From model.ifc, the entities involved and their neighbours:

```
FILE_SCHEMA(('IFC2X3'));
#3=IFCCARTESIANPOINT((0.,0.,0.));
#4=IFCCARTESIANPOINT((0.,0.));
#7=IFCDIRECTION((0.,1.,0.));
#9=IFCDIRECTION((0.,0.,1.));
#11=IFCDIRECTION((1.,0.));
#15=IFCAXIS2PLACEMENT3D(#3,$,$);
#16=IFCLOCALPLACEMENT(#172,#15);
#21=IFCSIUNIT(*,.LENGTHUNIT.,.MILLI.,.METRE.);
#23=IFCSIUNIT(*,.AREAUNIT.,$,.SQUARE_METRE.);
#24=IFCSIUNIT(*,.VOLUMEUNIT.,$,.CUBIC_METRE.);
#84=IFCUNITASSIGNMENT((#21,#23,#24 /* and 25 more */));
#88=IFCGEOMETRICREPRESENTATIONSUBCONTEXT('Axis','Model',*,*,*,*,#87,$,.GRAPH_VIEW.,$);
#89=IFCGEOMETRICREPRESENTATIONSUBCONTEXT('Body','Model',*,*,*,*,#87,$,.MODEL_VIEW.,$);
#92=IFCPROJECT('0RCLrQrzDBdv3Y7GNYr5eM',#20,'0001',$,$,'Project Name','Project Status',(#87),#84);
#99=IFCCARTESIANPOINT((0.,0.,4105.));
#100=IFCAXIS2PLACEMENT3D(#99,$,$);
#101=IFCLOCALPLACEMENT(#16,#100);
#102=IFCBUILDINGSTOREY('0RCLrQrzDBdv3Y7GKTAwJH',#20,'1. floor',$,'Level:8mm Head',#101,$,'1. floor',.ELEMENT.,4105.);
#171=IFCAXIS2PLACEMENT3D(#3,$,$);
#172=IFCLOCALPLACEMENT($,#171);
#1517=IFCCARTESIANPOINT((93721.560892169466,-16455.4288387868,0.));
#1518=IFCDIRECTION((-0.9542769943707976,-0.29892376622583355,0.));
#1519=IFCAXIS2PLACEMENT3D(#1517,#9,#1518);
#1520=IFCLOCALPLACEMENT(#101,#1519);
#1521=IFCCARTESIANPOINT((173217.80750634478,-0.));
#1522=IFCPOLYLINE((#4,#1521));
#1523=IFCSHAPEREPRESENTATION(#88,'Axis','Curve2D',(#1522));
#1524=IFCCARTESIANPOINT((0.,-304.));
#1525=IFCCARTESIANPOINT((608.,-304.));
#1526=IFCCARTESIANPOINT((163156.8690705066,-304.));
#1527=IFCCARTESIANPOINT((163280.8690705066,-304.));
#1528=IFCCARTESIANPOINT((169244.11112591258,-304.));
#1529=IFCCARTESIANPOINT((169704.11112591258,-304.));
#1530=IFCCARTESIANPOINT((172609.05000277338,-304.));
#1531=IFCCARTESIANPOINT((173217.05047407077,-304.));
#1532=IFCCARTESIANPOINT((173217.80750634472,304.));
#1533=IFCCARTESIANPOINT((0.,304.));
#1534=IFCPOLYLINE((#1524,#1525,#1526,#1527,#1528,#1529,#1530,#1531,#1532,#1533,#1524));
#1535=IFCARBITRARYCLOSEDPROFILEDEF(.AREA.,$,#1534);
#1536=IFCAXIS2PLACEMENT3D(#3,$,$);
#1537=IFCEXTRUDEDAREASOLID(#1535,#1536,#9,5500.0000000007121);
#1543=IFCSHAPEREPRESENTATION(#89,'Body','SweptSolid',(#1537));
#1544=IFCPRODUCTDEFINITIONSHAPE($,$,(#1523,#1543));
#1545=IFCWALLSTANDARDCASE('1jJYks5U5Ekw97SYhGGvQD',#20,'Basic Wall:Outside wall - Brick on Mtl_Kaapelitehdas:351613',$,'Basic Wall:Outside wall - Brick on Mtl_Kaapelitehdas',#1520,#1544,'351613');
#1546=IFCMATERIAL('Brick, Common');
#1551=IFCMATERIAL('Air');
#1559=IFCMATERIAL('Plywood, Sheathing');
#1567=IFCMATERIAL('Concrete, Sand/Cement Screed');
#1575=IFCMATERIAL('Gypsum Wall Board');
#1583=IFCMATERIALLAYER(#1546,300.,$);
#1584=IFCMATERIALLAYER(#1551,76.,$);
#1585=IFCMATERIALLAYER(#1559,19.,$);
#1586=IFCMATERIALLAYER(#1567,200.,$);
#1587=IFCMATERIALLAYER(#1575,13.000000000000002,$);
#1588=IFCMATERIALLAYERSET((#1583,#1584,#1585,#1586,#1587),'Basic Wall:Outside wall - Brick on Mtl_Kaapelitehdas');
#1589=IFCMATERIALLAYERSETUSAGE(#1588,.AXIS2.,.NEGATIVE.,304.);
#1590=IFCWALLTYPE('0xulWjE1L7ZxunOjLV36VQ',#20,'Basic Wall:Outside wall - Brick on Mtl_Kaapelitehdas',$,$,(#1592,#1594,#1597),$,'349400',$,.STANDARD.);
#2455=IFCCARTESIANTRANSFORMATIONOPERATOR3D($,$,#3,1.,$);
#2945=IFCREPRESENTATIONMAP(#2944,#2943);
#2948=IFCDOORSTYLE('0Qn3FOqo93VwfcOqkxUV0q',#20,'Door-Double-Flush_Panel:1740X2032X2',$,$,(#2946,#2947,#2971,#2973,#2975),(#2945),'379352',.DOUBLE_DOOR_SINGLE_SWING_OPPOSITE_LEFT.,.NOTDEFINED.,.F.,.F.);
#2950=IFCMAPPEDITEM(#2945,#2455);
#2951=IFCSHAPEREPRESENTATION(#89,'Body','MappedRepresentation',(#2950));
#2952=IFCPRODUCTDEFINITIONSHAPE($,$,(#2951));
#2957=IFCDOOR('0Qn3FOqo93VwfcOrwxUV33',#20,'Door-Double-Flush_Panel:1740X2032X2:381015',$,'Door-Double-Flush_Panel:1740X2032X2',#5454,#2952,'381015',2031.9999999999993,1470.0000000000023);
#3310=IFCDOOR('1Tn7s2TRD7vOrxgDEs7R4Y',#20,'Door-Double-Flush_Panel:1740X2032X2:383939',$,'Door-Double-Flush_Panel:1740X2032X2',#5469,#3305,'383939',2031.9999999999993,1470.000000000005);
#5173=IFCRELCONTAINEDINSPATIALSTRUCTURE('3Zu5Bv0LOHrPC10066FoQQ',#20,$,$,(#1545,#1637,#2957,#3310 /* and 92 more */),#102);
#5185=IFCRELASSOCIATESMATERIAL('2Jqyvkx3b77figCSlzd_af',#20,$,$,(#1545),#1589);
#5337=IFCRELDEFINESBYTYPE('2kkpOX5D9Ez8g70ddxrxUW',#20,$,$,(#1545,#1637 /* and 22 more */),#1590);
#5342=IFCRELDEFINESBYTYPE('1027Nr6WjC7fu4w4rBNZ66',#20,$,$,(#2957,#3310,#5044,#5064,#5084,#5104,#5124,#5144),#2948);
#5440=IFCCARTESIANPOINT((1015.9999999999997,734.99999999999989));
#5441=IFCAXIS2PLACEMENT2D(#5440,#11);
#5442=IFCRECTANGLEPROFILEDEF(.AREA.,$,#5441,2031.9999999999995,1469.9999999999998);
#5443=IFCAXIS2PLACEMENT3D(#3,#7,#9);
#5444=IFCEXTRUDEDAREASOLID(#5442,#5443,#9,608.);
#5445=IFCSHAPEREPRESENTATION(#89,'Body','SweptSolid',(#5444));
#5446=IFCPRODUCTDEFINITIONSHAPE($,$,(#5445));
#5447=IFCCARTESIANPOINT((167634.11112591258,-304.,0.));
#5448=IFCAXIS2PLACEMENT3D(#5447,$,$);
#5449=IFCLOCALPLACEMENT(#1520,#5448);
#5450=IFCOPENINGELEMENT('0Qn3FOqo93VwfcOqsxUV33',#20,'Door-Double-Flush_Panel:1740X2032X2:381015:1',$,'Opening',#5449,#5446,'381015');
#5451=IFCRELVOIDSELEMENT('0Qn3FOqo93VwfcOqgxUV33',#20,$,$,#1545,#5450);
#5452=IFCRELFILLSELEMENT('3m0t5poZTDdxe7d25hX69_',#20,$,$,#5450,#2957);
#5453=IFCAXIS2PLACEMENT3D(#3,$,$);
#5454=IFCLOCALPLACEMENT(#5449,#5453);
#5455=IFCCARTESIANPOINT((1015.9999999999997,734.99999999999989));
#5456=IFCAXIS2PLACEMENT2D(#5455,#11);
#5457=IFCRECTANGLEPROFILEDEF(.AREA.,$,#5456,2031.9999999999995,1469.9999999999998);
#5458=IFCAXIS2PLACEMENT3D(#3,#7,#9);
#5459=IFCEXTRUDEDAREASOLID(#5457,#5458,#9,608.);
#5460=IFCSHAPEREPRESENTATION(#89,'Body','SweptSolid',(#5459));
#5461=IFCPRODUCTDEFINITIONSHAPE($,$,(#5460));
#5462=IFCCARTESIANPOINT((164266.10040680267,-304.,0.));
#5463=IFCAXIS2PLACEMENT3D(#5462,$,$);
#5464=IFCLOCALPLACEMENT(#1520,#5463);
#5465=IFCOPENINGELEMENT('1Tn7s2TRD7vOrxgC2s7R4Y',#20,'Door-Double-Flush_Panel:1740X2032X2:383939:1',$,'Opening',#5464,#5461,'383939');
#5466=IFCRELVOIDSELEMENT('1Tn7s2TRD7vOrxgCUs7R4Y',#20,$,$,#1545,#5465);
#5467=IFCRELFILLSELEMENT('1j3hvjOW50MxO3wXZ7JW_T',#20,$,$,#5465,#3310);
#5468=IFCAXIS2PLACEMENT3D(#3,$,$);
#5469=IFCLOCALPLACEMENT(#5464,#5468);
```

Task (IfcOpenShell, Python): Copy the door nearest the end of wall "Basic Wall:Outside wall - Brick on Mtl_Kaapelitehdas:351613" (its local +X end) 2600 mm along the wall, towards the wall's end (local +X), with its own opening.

```python
import ifcopenshell
import ifcopenshell.api.feature
import ifcopenshell.api.geometry
import ifcopenshell.api.root
import ifcopenshell.geom
import ifcopenshell.util.element
import ifcopenshell.util.placement
import ifcopenshell.util.shape

model = ifcopenshell.open("model.ifc")
settings = ifcopenshell.geom.settings()


def volume(element):
    """Net volume in cubic metres, openings subtracted."""
    shape = ifcopenshell.geom.create_shape(settings, element)
    return ifcopenshell.util.shape.get_volume(shape.geometry)


def reuse_history(source, copy):
    """copy_class also copies each property set's owner history, people and application; keep the originals."""
    for rel in copy.IsDefinedBy:
        if rel.is_a("IfcRelDefinesByProperties") and (history := rel.RelatingPropertyDefinition.OwnerHistory):
            rel.RelatingPropertyDefinition.OwnerHistory = source.OwnerHistory
            ifcopenshell.util.element.remove_deep2(model, history)


door = model.by_guid("0Qn3FOqo93VwfcOrwxUV33")
opening = door.FillsVoids[0].RelatingOpeningElement
wall = opening.VoidsElements[0].RelatingBuildingElement
before = volume(wall)
shift = ifcopenshell.util.placement.get_local_placement(wall.ObjectPlacement)[:3, 0] * 2600.0

# copy_class copies the void relationship, type, container and properties, but no geometry.
new_opening = ifcopenshell.api.root.copy_class(model, product=opening)
new_opening.Representation = ifcopenshell.util.element.copy_deep(
    model, opening.Representation, exclude=["IfcGeometricRepresentationContext", "IfcRepresentationMap"]
)
new_opening.Name = "Door-Double-Flush_Panel:1740X2032X2"
new_opening.Tag = None
new_door = ifcopenshell.api.root.copy_class(model, product=door)
new_door.Representation = ifcopenshell.util.element.copy_deep(
    model, door.Representation, exclude=["IfcGeometricRepresentationContext", "IfcRepresentationMap"]
)
new_door.Name = "Door-Double-Flush_Panel:1740X2032X2"
new_door.Tag = None
reuse_history(door, new_door)
fills = ifcopenshell.api.feature.add_filling(model, opening=new_opening, element=new_door)
fills.OwnerHistory = new_door.OwnerHistory  # required in IFC2X3

for old, new in ((opening, new_opening), (door, new_door)):
    matrix = ifcopenshell.util.placement.get_local_placement(old.ObjectPlacement)
    matrix[:3, 3] += shift
    ifcopenshell.api.geometry.edit_object_placement(model, product=new, matrix=matrix, is_si=False)

after = volume(wall)

print(f"wall volume {before:.3f} -> {after:.3f} m3")

model.write("model_v2.ifc")
```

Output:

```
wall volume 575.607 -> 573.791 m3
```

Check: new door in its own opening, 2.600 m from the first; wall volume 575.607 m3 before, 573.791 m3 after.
